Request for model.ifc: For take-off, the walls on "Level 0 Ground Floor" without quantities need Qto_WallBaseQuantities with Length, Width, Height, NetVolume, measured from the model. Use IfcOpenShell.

First a look at what the model holds.

```python
import ifcopenshell
import ifcopenshell.util.element
import ifcopenshell.util.unit

model = ifcopenshell.open("model.ifc")
print(model.schema)
for unit_type in ("LENGTHUNIT", "AREAUNIT", "VOLUMEUNIT"):
    print(unit_type, ifcopenshell.util.unit.calculate_unit_scale(model, unit_type))
storey = next(s for s in model.by_type("IfcBuildingStorey") if s.Name == "Level 0 Ground Floor")
walls = [e for e in ifcopenshell.util.element.get_decomposition(storey) if e.is_a("IfcWall")]
for e in sorted(walls, key=lambda e: e.id()):
    print(e.id(), e.is_a(), e.Name, list(ifcopenshell.util.element.get_psets(e, qtos_only=True)), sep=" | ")
```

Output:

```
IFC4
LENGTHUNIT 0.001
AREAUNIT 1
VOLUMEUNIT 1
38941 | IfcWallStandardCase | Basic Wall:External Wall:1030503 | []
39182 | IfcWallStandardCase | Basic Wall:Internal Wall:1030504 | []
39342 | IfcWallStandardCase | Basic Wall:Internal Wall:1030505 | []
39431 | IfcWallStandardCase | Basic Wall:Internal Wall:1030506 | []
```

```python
import ifcopenshell
import ifcopenshell.api.pset
import ifcopenshell.geom
import ifcopenshell.util.element
import ifcopenshell.util.shape
import ifcopenshell.util.unit

model = ifcopenshell.open("model.ifc")
unit_scale = ifcopenshell.util.unit.calculate_unit_scale(model)
volume_scale = ifcopenshell.util.unit.calculate_unit_scale(model, "VOLUMEUNIT")
settings = ifcopenshell.geom.settings()

storey = next(s for s in model.by_type("IfcBuildingStorey") if s.Name == "Level 0 Ground Floor")
walls = [e for e in ifcopenshell.util.element.get_decomposition(storey) if e.is_a("IfcWall")]

for e in sorted(walls, key=lambda e: e.id()):
    if ifcopenshell.util.element.get_psets(e, qtos_only=True, should_inherit=False):
        continue
    # Geometry comes back in metres, in the element's own axes.
    shape = ifcopenshell.geom.create_shape(settings, e)
    values = {
        "Length": ifcopenshell.util.shape.get_x(shape.geometry) / unit_scale,
        "Width": ifcopenshell.util.shape.get_y(shape.geometry) / unit_scale,
        "Height": ifcopenshell.util.shape.get_z(shape.geometry) / unit_scale,
        "NetVolume": ifcopenshell.util.shape.get_volume(shape.geometry) / volume_scale,
    }
    qto = ifcopenshell.api.pset.add_qto(model, product=e, name="Qto_WallBaseQuantities")
    ifcopenshell.api.pset.edit_qto(model, qto=qto, properties=values)
    print(e.id(), {k: round(v, 3) for k, v in values.items()})

model.write("model-out.ifc")
```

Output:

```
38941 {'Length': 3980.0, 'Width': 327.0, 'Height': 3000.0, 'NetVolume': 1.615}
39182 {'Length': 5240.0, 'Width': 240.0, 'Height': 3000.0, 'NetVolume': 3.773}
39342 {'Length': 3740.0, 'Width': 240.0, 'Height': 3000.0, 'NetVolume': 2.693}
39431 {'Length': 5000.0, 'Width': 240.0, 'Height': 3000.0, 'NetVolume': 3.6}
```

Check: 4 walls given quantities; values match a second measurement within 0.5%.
